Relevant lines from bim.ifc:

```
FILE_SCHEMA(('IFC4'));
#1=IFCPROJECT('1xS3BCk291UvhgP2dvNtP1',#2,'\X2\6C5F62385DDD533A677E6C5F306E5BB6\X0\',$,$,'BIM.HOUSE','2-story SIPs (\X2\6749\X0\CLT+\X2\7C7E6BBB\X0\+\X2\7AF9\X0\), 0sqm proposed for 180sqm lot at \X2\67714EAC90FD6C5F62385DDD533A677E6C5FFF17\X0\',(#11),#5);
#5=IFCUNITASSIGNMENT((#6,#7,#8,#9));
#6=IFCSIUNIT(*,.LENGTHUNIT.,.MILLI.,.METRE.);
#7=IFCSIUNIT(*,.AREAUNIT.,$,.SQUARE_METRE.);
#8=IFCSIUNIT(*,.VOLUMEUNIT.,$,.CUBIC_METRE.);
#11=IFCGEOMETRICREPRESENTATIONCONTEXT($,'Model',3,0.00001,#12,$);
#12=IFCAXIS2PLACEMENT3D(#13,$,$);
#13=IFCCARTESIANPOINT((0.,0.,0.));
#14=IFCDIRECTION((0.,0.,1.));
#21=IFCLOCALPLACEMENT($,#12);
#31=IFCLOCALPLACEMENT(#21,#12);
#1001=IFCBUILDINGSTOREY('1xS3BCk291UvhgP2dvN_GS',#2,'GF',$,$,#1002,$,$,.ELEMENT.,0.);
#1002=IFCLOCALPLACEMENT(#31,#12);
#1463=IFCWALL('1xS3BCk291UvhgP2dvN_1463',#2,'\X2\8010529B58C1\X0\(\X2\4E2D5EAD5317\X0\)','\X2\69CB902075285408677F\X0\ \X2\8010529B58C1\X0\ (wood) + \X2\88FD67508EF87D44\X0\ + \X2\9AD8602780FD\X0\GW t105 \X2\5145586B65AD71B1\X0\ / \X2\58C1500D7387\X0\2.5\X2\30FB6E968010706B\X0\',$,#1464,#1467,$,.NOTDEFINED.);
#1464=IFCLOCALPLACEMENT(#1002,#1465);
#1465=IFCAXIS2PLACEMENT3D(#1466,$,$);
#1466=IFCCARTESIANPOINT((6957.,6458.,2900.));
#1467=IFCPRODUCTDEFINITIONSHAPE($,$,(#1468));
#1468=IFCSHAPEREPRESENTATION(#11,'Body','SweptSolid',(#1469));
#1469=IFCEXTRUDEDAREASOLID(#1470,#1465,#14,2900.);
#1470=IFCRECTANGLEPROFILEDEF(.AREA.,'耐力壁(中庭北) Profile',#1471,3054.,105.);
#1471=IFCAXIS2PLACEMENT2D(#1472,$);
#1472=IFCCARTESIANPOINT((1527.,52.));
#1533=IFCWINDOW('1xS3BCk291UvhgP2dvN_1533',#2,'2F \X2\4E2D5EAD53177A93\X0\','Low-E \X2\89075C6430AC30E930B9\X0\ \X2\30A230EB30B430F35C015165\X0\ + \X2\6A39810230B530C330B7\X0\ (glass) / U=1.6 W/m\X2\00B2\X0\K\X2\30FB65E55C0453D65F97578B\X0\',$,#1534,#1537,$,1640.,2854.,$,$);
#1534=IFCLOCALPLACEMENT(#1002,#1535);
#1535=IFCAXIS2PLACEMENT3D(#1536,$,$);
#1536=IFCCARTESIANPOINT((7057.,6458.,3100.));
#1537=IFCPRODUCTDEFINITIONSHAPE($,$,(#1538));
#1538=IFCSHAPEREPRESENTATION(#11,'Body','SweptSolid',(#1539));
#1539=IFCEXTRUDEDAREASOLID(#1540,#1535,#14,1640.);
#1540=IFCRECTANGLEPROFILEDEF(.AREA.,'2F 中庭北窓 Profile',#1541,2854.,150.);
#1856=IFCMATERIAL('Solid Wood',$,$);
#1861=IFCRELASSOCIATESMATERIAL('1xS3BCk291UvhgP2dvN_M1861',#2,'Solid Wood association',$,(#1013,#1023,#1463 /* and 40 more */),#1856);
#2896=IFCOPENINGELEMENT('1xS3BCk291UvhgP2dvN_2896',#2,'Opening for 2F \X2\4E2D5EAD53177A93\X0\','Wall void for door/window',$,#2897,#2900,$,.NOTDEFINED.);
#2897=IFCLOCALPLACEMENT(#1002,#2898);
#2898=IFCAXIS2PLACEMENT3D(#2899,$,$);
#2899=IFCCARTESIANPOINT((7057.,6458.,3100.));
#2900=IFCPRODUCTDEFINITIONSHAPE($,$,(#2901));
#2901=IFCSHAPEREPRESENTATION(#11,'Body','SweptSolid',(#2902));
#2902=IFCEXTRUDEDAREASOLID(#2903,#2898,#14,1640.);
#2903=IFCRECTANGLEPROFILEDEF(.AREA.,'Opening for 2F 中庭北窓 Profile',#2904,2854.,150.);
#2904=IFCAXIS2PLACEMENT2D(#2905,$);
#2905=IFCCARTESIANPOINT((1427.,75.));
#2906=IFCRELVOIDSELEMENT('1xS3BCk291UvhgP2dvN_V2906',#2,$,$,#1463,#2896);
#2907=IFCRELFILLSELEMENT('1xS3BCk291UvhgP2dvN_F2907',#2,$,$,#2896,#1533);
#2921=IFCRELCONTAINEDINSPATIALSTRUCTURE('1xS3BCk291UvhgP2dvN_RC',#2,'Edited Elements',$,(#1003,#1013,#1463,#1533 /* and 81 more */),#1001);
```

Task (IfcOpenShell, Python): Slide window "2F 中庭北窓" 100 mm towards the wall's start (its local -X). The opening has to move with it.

```python
import ifcopenshell
import ifcopenshell.api.geometry
import ifcopenshell.util.placement
import ifcopenshell.util.unit

model = ifcopenshell.open("bim.ifc")
unit_scale = ifcopenshell.util.unit.calculate_unit_scale(model)

window = model.by_guid("1xS3BCk291UvhgP2dvN_1533")
opening = window.FillsVoids[0].RelatingOpeningElement
wall = opening.VoidsElements[0].RelatingBuildingElement

wall_matrix = ifcopenshell.util.placement.get_local_placement(wall.ObjectPlacement)
shift = wall_matrix[:3, 0] * -0.1 / unit_scale
before = ifcopenshell.util.placement.get_local_placement(window.ObjectPlacement)[:3, 3].copy()

# The window is not placed relative to its opening, so move both.
for product in (opening, window):
    matrix = ifcopenshell.util.placement.get_local_placement(product.ObjectPlacement)
    matrix[:3, 3] += shift
    ifcopenshell.api.geometry.edit_object_placement(model, product=product, matrix=matrix, is_si=False)

after = ifcopenshell.util.placement.get_local_placement(window.ObjectPlacement)[:3, 3]
print("window moved by", (after - before).round(3) + 0.0)

model.write("bim_rev.ifc")
```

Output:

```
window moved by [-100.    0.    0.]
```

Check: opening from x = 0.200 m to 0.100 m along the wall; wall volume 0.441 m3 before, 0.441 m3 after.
